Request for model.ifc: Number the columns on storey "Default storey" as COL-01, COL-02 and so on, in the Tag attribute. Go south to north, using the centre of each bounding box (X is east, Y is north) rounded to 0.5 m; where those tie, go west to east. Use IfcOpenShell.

First a look at what the model holds.

```python
import ifcopenshell
import ifcopenshell.util.element
import ifcopenshell.util.placement

model = ifcopenshell.open("model.ifc")
print(model.schema)
storey = next(s for s in model.by_type("IfcBuildingStorey") if s.Name == "Default storey")
columns = [e for e in ifcopenshell.util.element.get_decomposition(storey) if e.is_a("IfcColumn")]
for e in sorted(columns, key=lambda e: e.id()):
    origin = ifcopenshell.util.placement.get_local_placement(e.ObjectPlacement)[:3, 3]
    print(e.id(), e.Tag, e.Name, origin.round(2) + 0.0, sep=" | ")
```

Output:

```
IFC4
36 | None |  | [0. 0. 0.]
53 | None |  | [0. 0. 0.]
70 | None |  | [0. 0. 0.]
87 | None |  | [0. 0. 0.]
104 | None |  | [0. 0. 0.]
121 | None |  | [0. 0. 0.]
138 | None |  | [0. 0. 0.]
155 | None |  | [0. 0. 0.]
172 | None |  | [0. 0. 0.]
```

```python
import ifcopenshell
import ifcopenshell.geom
import ifcopenshell.util.element
import ifcopenshell.util.shape

model = ifcopenshell.open("model.ifc")
settings = ifcopenshell.geom.settings()
settings.set("use-world-coords", True)


def centre(element):
    shape = ifcopenshell.geom.create_shape(settings, element)
    return ifcopenshell.util.shape.get_bbox_centroid(shape.geometry)


storey = next(s for s in model.by_type("IfcBuildingStorey") if s.Name == "Default storey")
columns = [e for e in ifcopenshell.util.element.get_decomposition(storey) if e.is_a("IfcColumn")]

# Insertion points can sit at a corner or the storey origin, so sort by the geometry (in metres).
centres = {e: centre(e) for e in columns}
columns.sort(key=lambda e: (round(centres[e][1] / 0.5), centres[e][0]))

for i, e in enumerate(columns, start=1):
    number = f"COL-{i:02d}"
    e.Tag = number
    print(e.id(), number)

model.write("model_updated.ifc")
```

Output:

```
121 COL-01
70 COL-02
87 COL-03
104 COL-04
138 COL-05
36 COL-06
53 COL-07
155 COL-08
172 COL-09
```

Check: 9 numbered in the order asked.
